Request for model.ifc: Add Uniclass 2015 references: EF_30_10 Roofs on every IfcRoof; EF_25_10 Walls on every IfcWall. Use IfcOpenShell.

First a look at what the model holds.

```python
import ifcopenshell

model = ifcopenshell.open("model.ifc")
print(model.schema)
print("classifications:", [c.Name for c in model.by_type("IfcClassification")])
for ifc_class in ("IfcDoor", "IfcRoof", "IfcStair", "IfcWall", "IfcWindow"):
    print(ifc_class, len(model.by_type(ifc_class)))
```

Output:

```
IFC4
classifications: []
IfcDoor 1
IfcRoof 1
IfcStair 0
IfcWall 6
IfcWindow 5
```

```python
import ifcopenshell
import ifcopenshell.api.classification

model = ifcopenshell.open("model.ifc")

system = ifcopenshell.api.classification.add_classification(model, classification="Uniclass 2015")

codes = {
    "IfcRoof": ("EF_30_10", "Roofs"),
    "IfcWall": ("EF_25_10", "Walls"),
}
for ifc_class, (code, name) in codes.items():
    products = model.by_type(ifc_class)
    ifcopenshell.api.classification.add_reference(
        model, products=products, classification=system, identification=code, name=name
    )
    print(code, len(products))

model.write("model_rev.ifc")
```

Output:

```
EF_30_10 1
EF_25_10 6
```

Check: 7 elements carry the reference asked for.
